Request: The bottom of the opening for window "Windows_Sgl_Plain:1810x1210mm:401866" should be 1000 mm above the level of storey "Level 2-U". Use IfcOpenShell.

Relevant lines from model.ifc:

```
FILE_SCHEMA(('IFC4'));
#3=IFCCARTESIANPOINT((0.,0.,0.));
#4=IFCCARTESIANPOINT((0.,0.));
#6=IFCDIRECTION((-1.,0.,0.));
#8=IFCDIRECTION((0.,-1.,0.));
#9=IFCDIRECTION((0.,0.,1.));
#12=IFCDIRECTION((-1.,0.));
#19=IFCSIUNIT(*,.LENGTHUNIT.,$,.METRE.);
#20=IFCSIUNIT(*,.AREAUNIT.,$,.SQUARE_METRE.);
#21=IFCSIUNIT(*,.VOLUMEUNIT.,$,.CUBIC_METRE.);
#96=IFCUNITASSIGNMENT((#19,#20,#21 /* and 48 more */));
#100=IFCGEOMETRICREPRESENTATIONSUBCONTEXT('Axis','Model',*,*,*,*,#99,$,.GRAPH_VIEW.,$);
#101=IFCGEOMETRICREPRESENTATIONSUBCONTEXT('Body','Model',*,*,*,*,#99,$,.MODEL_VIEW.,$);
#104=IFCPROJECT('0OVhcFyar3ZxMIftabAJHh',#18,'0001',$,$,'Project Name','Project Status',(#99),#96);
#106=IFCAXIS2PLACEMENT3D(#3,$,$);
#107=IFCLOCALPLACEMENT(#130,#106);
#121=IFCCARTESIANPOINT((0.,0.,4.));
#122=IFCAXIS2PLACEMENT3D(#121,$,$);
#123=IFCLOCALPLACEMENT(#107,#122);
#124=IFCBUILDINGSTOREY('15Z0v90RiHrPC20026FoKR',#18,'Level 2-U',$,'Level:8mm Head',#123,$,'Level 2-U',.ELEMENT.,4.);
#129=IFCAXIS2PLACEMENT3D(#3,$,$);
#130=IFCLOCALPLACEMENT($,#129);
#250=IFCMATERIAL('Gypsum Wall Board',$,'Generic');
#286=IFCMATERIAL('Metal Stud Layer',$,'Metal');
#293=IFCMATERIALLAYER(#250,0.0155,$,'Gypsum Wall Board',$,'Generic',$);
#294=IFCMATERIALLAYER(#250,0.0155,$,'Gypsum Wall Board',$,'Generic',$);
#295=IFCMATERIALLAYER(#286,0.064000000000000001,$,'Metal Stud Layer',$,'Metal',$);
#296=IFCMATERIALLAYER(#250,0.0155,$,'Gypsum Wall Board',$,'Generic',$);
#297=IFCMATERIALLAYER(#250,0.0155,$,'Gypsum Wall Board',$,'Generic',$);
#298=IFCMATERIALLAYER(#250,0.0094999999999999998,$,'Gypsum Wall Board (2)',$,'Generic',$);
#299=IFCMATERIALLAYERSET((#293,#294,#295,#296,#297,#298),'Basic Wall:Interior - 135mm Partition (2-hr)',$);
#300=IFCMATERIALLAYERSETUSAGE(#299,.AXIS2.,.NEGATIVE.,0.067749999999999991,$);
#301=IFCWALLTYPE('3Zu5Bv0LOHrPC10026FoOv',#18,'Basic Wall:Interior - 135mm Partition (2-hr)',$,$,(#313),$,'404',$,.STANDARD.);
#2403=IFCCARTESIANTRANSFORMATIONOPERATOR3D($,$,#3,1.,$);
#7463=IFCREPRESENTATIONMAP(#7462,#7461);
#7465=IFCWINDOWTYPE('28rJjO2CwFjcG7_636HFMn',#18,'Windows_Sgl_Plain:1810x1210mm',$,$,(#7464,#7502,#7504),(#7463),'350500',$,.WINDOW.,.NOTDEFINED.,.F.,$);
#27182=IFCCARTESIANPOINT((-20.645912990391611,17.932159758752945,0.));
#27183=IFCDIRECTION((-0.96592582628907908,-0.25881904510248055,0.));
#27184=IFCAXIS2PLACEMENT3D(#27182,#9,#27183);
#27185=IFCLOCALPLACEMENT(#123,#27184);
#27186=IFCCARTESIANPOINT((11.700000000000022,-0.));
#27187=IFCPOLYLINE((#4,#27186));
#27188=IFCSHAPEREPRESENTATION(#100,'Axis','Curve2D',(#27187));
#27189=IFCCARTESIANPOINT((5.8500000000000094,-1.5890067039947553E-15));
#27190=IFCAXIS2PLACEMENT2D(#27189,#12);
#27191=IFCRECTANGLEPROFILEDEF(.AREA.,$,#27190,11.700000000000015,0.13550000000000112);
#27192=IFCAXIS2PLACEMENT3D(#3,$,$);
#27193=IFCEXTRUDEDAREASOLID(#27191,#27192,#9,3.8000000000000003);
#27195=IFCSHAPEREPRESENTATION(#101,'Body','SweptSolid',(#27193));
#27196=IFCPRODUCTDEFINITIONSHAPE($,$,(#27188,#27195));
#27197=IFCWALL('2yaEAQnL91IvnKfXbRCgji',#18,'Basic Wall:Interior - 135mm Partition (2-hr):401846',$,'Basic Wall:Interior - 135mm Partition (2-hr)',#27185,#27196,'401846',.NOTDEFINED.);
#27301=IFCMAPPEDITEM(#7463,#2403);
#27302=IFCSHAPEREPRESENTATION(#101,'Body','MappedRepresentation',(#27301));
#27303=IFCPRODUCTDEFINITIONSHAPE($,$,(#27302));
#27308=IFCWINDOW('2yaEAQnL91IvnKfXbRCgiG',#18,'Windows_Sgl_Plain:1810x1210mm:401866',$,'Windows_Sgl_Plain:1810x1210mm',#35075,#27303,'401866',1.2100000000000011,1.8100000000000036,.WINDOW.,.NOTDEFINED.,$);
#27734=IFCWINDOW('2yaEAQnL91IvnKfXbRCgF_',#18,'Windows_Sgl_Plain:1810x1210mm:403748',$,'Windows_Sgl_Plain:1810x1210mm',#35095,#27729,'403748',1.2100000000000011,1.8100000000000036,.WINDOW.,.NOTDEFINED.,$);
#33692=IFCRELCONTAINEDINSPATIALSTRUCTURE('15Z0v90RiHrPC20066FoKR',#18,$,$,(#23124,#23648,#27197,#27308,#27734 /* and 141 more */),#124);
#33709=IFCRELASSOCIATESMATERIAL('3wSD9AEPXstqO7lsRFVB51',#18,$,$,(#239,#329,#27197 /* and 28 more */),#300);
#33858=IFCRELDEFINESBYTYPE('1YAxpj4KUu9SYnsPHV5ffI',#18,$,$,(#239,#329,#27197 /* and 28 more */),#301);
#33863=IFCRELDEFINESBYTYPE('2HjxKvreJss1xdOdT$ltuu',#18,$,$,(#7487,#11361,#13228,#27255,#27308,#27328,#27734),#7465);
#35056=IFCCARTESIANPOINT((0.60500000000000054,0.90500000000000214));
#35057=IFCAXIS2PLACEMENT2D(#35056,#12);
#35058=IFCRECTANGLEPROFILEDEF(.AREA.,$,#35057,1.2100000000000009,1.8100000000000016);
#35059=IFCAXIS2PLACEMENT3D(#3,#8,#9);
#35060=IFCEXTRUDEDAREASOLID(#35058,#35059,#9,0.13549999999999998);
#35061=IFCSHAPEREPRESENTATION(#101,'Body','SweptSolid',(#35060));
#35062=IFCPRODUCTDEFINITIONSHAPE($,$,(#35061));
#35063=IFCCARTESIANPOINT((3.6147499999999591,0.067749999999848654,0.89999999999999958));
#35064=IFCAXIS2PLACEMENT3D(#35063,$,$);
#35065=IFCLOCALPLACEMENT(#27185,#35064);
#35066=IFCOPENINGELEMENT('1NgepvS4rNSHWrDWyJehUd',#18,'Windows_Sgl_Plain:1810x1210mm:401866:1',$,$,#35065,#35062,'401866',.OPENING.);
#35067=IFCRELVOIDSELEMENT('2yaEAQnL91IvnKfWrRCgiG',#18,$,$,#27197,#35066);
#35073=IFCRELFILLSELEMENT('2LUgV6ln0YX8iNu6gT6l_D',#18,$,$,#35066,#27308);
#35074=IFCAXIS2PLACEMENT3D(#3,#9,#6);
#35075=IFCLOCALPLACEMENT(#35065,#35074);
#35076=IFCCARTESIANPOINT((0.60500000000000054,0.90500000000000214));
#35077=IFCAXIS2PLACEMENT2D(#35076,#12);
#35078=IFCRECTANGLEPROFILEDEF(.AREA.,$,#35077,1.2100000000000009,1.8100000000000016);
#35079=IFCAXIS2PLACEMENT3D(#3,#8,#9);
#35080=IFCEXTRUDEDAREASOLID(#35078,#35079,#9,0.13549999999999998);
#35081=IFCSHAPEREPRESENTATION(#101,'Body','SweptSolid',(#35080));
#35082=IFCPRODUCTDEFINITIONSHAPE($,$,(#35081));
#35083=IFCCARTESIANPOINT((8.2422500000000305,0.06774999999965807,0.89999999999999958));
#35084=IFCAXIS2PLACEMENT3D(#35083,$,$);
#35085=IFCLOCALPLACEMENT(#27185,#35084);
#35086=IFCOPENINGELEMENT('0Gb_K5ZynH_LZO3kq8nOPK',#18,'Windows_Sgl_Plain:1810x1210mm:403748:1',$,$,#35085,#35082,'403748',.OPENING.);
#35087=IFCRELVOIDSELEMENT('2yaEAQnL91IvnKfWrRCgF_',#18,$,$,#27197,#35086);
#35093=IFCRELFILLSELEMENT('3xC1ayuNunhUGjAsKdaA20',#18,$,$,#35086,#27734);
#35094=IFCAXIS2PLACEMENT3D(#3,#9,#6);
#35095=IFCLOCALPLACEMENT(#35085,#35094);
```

```python
import numpy as np
import ifcopenshell
import ifcopenshell.api.geometry
import ifcopenshell.geom
import ifcopenshell.util.element
import ifcopenshell.util.placement
import ifcopenshell.util.shape
import ifcopenshell.util.unit

model = ifcopenshell.open("model.ifc")
unit_scale = ifcopenshell.util.unit.calculate_unit_scale(model)

window = model.by_id(27308)
opening = window.FillsVoids[0].RelatingOpeningElement
storey = ifcopenshell.util.element.get_container(window, ifc_class="IfcBuildingStorey")
level = ifcopenshell.util.placement.get_local_placement(storey.ObjectPlacement)[2, 3]

# The opening's origin need not be at the sill, so measure its lowest point.
shape = ifcopenshell.geom.create_shape(ifcopenshell.geom.settings(), opening)
bottom = ifcopenshell.util.shape.get_shape_bottom_elevation(shape, shape.geometry) / unit_scale
dz = level + 1.0 - bottom

shift = np.array([0.0, 0.0, dz])
# The window is placed relative to its opening, so it follows when the opening moves.
matrix = ifcopenshell.util.placement.get_local_placement(opening.ObjectPlacement)
matrix[:3, 3] += shift
ifcopenshell.api.geometry.edit_object_placement(
    model, product=opening, matrix=matrix, is_si=False, should_transform_children=True
)

print(f"moved by {dz * unit_scale:+.3f} m")

model.write("model_edited.ifc")
```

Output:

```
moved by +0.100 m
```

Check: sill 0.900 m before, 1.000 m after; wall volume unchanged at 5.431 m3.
